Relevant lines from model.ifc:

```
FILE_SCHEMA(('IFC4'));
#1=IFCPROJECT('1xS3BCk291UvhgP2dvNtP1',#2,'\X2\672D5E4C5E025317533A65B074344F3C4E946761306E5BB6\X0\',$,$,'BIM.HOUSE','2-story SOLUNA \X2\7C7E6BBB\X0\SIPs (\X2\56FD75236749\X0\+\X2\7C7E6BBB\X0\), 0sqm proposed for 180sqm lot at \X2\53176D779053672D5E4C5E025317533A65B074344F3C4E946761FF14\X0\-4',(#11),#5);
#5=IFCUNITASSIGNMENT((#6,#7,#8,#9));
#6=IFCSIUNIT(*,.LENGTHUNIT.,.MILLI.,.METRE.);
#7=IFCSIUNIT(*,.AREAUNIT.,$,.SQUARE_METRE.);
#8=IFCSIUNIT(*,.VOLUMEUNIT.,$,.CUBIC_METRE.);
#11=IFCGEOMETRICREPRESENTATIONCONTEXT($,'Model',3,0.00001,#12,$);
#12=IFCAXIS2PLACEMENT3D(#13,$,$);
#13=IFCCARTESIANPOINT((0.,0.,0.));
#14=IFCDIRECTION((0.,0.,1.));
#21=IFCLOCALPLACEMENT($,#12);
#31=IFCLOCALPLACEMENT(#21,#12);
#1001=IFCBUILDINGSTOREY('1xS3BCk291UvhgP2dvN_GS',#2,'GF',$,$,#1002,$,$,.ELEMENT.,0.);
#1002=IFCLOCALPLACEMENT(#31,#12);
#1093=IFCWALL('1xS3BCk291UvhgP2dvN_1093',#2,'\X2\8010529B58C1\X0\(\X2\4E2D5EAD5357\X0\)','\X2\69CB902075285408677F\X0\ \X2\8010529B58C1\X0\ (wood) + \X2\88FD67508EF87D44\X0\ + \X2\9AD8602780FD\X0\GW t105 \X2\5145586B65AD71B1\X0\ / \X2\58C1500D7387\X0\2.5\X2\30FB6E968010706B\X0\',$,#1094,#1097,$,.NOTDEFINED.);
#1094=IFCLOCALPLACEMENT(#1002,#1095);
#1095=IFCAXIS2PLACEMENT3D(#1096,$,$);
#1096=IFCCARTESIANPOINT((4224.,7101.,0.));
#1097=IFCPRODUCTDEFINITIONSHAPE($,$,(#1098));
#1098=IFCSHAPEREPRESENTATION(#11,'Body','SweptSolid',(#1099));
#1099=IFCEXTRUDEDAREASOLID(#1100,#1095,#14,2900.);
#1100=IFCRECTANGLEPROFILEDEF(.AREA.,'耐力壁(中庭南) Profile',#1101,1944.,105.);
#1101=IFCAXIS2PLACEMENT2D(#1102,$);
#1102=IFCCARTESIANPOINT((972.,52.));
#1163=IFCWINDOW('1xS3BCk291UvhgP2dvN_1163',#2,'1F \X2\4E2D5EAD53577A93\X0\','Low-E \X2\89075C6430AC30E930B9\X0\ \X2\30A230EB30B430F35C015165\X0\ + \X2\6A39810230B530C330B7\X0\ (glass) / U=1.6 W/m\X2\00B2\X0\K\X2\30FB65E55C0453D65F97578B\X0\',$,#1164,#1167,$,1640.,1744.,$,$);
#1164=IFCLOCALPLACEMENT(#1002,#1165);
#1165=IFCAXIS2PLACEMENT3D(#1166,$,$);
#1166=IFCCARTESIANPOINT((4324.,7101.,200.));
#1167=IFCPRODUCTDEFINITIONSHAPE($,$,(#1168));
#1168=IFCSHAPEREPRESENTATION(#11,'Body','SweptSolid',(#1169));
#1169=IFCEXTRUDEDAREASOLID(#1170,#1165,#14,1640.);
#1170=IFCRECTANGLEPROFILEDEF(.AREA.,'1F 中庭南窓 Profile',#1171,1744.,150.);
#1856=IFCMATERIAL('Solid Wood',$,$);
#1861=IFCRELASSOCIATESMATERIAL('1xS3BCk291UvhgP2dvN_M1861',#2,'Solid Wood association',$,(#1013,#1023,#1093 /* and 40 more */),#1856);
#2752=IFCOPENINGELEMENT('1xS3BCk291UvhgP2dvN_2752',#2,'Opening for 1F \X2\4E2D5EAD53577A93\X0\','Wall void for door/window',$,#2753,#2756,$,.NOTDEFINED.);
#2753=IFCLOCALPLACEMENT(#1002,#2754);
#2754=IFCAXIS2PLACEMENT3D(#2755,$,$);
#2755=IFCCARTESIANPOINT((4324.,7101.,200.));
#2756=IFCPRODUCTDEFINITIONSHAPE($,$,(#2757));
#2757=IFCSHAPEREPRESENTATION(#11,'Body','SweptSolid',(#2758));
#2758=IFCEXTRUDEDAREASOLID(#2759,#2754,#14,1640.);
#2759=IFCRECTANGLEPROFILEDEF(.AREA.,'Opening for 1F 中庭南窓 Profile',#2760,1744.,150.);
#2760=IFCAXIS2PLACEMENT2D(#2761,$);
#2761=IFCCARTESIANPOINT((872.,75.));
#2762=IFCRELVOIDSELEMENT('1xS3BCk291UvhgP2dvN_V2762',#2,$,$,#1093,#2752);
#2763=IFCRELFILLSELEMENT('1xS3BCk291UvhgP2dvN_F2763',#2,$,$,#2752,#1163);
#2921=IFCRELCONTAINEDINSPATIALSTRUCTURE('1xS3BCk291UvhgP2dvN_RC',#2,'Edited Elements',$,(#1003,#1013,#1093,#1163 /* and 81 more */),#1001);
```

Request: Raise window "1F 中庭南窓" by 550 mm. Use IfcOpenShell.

```python
import numpy as np
import ifcopenshell
import ifcopenshell.api.geometry
import ifcopenshell.util.placement
import ifcopenshell.util.unit

model = ifcopenshell.open("model.ifc")
unit_scale = ifcopenshell.util.unit.calculate_unit_scale(model)

window = model.by_id(1163)
opening = window.FillsVoids[0].RelatingOpeningElement
dz = 0.55 / unit_scale

shift = np.array([0.0, 0.0, dz])
# The window is not placed relative to its opening, so move both.
for product in (opening, window):
    matrix = ifcopenshell.util.placement.get_local_placement(product.ObjectPlacement)
    matrix[:3, 3] += shift
    ifcopenshell.api.geometry.edit_object_placement(model, product=product, matrix=matrix, is_si=False)

print(f"moved by {dz * unit_scale:+.3f} m")

model.write("model-out.ifc")
```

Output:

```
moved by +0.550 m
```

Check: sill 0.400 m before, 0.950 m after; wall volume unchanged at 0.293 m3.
